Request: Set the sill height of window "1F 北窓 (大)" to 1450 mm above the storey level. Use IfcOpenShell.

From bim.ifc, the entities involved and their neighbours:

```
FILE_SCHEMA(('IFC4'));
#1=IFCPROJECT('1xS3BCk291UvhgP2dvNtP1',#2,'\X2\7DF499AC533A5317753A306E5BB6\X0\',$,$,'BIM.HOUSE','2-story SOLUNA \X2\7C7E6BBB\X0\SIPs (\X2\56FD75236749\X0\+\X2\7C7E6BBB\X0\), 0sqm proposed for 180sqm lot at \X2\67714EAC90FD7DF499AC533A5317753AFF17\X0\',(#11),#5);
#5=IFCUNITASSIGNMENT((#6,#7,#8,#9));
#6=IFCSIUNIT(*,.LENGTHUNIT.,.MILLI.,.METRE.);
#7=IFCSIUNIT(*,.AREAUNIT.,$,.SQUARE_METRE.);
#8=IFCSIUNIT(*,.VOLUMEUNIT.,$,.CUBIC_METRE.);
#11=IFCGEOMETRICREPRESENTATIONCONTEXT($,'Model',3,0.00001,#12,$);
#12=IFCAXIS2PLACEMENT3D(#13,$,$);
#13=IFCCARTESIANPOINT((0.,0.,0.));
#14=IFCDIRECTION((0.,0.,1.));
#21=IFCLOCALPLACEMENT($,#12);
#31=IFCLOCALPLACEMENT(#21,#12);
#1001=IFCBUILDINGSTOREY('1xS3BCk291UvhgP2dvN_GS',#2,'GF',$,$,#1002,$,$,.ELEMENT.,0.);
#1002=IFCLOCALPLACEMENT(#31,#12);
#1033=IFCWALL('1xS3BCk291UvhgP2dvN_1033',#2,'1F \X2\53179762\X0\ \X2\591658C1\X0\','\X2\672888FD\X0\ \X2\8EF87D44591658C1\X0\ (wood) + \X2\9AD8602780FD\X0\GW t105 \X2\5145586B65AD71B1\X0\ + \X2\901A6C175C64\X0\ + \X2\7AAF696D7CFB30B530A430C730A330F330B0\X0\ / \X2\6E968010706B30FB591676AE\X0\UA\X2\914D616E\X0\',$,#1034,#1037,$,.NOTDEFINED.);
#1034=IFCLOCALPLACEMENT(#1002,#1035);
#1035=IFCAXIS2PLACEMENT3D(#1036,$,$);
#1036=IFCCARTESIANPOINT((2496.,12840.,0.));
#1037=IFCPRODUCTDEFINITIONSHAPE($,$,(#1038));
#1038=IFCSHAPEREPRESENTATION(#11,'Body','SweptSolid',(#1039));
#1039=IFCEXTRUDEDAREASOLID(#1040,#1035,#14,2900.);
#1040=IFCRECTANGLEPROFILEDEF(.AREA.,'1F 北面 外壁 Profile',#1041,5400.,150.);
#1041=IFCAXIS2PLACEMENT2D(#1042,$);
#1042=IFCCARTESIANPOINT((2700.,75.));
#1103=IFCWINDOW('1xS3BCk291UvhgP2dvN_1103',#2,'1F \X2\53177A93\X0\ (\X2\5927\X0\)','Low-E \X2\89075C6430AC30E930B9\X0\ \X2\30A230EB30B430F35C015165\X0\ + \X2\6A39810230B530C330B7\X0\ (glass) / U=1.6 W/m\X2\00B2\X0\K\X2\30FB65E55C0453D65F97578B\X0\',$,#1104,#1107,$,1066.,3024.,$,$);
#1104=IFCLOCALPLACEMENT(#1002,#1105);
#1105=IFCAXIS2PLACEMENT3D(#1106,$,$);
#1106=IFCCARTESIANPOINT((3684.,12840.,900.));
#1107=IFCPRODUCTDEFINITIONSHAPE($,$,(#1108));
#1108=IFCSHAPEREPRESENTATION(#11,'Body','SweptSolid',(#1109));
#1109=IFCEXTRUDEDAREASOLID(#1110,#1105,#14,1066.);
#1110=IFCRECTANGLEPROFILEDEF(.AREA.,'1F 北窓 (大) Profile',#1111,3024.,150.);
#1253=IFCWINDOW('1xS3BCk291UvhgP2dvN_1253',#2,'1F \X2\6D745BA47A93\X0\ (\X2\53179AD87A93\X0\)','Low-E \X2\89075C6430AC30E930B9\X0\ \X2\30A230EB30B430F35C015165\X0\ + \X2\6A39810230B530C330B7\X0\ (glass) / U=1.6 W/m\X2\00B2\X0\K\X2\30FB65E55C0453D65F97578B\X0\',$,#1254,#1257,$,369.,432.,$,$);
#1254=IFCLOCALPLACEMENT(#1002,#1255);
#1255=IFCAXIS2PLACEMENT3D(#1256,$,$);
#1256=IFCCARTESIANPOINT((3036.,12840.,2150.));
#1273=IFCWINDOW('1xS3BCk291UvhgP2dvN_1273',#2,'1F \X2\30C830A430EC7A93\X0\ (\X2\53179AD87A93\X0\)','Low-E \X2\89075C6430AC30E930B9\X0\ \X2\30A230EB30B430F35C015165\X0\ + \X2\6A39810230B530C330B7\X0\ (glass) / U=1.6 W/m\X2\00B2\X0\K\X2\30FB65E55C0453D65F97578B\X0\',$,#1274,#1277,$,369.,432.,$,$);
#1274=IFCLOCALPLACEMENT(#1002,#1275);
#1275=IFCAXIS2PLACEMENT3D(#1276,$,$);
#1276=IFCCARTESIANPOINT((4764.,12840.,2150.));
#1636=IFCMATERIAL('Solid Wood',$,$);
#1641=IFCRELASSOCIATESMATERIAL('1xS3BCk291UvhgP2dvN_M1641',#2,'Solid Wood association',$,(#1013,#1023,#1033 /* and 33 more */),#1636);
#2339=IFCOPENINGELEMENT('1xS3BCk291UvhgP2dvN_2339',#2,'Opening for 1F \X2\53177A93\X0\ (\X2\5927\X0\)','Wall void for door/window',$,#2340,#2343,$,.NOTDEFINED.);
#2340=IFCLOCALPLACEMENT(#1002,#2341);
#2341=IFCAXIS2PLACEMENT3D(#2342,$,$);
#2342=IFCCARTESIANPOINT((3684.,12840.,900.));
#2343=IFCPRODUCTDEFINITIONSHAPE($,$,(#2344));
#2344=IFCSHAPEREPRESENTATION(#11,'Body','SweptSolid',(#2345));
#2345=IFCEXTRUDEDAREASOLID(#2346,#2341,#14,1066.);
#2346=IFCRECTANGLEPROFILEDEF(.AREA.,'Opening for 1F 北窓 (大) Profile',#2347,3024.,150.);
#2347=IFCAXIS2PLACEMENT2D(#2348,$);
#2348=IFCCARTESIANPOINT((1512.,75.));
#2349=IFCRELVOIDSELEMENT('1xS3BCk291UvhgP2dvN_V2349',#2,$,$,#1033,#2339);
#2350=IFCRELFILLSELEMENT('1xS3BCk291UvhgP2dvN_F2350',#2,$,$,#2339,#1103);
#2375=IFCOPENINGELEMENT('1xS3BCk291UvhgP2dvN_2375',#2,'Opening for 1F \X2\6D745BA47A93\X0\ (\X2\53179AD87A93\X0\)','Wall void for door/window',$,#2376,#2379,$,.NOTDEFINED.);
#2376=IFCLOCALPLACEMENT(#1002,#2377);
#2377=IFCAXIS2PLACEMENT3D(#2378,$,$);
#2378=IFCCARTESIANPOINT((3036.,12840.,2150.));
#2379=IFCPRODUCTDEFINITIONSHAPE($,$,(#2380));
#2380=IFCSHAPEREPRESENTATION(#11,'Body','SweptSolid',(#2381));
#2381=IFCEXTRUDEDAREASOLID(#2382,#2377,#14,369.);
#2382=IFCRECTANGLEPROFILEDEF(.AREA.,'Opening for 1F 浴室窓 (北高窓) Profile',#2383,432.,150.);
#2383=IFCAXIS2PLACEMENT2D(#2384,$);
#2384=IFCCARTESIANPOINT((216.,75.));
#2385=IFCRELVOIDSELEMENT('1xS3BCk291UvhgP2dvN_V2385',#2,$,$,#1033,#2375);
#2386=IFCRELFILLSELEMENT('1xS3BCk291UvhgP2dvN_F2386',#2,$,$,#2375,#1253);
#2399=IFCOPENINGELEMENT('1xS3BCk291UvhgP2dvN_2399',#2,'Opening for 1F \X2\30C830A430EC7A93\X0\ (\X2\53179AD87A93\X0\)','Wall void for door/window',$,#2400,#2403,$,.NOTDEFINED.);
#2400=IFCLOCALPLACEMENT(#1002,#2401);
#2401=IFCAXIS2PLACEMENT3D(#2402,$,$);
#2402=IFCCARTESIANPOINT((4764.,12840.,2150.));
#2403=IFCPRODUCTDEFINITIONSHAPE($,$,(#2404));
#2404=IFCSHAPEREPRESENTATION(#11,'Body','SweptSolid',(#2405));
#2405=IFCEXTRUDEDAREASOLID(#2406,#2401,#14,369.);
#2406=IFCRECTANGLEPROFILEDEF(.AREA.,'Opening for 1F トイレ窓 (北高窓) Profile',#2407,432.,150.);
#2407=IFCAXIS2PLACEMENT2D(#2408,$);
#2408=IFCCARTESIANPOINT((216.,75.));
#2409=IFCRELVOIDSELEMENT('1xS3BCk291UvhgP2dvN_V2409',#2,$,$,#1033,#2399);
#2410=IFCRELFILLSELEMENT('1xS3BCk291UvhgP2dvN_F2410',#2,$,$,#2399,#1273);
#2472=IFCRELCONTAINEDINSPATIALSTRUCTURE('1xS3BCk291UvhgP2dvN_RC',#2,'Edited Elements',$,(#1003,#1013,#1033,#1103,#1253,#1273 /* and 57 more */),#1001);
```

```python
import numpy as np
import ifcopenshell
import ifcopenshell.api.geometry
import ifcopenshell.geom
import ifcopenshell.util.element
import ifcopenshell.util.placement
import ifcopenshell.util.shape
import ifcopenshell.util.unit

model = ifcopenshell.open("bim.ifc")
unit_scale = ifcopenshell.util.unit.calculate_unit_scale(model)

window = model.by_guid("1xS3BCk291UvhgP2dvN_1103")
opening = window.FillsVoids[0].RelatingOpeningElement
storey = ifcopenshell.util.element.get_container(window, ifc_class="IfcBuildingStorey")
level = ifcopenshell.util.placement.get_local_placement(storey.ObjectPlacement)[2, 3]

# The opening's origin need not be at the sill, so measure its lowest point.
shape = ifcopenshell.geom.create_shape(ifcopenshell.geom.settings(), opening)
bottom = ifcopenshell.util.shape.get_shape_bottom_elevation(shape, shape.geometry) / unit_scale
dz = level + 1450.0 - bottom

shift = np.array([0.0, 0.0, dz])
# The window is not placed relative to its opening, so move both.
for product in (opening, window):
    matrix = ifcopenshell.util.placement.get_local_placement(product.ObjectPlacement)
    matrix[:3, 3] += shift
    ifcopenshell.api.geometry.edit_object_placement(model, product=product, matrix=matrix, is_si=False)

print(f"moved by {dz * unit_scale:+.3f} m")

model.write("bim_v2.ifc")
```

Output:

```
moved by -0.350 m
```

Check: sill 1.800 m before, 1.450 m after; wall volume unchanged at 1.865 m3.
